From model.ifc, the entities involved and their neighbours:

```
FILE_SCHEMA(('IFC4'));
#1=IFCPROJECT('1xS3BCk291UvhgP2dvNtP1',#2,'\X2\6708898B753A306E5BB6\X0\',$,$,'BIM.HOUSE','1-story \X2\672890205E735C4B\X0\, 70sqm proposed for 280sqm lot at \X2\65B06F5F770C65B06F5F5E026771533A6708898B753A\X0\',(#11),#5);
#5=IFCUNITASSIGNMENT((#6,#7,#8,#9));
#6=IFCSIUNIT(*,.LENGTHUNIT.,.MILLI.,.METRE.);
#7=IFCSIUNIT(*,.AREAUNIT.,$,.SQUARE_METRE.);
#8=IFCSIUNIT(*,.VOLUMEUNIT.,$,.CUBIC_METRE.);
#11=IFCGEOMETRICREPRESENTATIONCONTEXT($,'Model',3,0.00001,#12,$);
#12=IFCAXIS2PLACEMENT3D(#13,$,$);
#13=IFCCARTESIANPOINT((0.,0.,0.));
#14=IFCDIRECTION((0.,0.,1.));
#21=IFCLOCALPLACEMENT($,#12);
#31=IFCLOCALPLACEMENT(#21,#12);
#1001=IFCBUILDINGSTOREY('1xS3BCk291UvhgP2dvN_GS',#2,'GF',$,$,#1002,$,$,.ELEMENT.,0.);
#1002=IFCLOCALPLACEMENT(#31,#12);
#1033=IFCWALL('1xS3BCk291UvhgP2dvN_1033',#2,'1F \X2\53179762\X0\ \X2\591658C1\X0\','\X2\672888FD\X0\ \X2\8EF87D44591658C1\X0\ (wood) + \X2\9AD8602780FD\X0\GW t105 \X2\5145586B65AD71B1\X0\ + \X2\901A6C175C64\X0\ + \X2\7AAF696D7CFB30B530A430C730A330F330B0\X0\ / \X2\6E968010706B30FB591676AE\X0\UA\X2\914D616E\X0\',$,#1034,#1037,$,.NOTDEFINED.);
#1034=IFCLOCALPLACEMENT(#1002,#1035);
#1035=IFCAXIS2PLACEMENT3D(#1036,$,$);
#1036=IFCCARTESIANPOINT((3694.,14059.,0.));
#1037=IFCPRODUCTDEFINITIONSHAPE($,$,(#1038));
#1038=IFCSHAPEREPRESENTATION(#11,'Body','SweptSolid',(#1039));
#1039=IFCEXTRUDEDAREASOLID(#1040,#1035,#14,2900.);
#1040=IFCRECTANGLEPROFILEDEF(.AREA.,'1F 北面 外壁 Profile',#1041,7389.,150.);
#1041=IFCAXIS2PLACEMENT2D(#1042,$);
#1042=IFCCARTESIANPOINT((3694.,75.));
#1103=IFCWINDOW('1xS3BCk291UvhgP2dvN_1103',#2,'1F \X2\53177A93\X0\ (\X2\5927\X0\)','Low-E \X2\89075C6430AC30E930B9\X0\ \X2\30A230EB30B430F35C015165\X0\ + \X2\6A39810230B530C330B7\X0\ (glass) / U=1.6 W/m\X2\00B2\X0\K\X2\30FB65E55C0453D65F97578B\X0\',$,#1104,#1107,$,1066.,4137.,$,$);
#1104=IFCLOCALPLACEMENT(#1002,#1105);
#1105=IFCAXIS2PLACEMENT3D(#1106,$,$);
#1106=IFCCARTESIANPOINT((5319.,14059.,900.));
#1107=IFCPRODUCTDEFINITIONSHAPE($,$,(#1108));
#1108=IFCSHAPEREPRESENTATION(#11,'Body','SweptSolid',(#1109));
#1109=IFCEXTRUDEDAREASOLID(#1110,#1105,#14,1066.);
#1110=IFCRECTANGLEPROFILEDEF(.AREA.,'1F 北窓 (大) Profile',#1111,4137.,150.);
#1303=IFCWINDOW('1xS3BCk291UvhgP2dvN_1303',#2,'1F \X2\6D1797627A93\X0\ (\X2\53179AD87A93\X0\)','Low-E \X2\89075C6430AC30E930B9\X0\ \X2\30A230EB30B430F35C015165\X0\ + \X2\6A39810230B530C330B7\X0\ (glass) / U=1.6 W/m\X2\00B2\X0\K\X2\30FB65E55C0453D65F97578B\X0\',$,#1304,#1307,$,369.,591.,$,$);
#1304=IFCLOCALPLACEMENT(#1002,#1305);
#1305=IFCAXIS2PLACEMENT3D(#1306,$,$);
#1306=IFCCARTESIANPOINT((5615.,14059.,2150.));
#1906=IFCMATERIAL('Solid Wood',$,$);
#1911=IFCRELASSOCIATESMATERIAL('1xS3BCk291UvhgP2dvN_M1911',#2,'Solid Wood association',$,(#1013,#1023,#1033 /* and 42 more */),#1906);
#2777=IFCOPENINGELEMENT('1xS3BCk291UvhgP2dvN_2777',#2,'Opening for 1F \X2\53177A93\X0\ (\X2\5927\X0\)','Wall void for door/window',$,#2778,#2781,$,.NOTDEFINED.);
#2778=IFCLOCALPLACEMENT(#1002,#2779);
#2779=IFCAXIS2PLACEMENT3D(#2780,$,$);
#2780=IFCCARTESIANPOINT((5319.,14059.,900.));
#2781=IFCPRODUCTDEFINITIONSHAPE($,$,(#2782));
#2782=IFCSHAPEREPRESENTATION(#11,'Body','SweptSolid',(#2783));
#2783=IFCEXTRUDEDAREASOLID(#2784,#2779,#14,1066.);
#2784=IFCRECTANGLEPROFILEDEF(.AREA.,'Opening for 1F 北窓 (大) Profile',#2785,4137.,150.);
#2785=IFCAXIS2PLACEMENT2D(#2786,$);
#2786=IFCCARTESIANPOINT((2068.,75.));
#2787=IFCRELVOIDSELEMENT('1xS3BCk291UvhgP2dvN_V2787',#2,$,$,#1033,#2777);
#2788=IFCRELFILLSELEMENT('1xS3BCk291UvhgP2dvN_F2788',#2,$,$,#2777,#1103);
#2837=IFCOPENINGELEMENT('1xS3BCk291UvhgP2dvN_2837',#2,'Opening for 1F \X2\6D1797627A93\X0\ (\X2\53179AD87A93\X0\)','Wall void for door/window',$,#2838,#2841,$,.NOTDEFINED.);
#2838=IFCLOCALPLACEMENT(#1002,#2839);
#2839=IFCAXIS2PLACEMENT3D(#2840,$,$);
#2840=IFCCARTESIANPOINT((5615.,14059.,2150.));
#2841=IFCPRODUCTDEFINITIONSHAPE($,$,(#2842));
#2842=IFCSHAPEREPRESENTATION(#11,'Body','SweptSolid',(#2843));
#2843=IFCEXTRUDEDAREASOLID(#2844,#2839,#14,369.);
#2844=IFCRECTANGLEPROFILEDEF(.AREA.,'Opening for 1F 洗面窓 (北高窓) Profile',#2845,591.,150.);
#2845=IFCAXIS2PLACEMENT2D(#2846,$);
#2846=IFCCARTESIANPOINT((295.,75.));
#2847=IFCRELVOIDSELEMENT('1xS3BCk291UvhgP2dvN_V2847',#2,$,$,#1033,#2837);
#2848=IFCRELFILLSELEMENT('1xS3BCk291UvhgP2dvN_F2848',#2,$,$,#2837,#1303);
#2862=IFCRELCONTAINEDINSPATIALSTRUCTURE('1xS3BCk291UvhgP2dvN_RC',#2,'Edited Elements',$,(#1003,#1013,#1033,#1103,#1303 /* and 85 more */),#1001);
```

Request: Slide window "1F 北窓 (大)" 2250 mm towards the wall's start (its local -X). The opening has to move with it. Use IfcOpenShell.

```python
import ifcopenshell
import ifcopenshell.api.geometry
import ifcopenshell.util.placement

model = ifcopenshell.open("model.ifc")

window = model.by_guid("1xS3BCk291UvhgP2dvN_1103")
opening = window.FillsVoids[0].RelatingOpeningElement
wall = opening.VoidsElements[0].RelatingBuildingElement

wall_matrix = ifcopenshell.util.placement.get_local_placement(wall.ObjectPlacement)
shift = wall_matrix[:3, 0] * -2250.0
before = ifcopenshell.util.placement.get_local_placement(window.ObjectPlacement)[:3, 3].copy()

# The window is not placed relative to its opening, so move both.
for product in (opening, window):
    matrix = ifcopenshell.util.placement.get_local_placement(product.ObjectPlacement)
    matrix[:3, 3] += shift
    ifcopenshell.api.geometry.edit_object_placement(model, product=product, matrix=matrix, is_si=False)

after = ifcopenshell.util.placement.get_local_placement(window.ObjectPlacement)[:3, 3]
print("window moved by", (after - before).round(3) + 0.0)

model.write("model_rev.ifc")
```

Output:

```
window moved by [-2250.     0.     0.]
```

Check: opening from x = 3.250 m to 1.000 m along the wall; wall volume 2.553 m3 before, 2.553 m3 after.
